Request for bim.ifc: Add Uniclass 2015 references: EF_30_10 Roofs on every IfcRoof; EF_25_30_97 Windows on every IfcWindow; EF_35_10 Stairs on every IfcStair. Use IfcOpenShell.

First a look at what the model holds.

```python
import ifcopenshell

model = ifcopenshell.open("bim.ifc")
print(model.schema)
print("classifications:", [c.Name for c in model.by_type("IfcClassification")])
for ifc_class in ("IfcDoor", "IfcRoof", "IfcStair", "IfcWall", "IfcWindow"):
    print(ifc_class, len(model.by_type(ifc_class)))
```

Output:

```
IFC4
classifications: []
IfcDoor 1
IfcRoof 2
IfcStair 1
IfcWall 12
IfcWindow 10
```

```python
import ifcopenshell
import ifcopenshell.api.classification

model = ifcopenshell.open("bim.ifc")

system = ifcopenshell.api.classification.add_classification(model, classification="Uniclass 2015")

codes = {
    "IfcRoof": ("EF_30_10", "Roofs"),
    "IfcWindow": ("EF_25_30_97", "Windows"),
    "IfcStair": ("EF_35_10", "Stairs"),
}
for ifc_class, (code, name) in codes.items():
    products = model.by_type(ifc_class)
    ifcopenshell.api.classification.add_reference(
        model, products=products, classification=system, identification=code, name=name
    )
    print(code, len(products))

model.write("bim-out.ifc")
```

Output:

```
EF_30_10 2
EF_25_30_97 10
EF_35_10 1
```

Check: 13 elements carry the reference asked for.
